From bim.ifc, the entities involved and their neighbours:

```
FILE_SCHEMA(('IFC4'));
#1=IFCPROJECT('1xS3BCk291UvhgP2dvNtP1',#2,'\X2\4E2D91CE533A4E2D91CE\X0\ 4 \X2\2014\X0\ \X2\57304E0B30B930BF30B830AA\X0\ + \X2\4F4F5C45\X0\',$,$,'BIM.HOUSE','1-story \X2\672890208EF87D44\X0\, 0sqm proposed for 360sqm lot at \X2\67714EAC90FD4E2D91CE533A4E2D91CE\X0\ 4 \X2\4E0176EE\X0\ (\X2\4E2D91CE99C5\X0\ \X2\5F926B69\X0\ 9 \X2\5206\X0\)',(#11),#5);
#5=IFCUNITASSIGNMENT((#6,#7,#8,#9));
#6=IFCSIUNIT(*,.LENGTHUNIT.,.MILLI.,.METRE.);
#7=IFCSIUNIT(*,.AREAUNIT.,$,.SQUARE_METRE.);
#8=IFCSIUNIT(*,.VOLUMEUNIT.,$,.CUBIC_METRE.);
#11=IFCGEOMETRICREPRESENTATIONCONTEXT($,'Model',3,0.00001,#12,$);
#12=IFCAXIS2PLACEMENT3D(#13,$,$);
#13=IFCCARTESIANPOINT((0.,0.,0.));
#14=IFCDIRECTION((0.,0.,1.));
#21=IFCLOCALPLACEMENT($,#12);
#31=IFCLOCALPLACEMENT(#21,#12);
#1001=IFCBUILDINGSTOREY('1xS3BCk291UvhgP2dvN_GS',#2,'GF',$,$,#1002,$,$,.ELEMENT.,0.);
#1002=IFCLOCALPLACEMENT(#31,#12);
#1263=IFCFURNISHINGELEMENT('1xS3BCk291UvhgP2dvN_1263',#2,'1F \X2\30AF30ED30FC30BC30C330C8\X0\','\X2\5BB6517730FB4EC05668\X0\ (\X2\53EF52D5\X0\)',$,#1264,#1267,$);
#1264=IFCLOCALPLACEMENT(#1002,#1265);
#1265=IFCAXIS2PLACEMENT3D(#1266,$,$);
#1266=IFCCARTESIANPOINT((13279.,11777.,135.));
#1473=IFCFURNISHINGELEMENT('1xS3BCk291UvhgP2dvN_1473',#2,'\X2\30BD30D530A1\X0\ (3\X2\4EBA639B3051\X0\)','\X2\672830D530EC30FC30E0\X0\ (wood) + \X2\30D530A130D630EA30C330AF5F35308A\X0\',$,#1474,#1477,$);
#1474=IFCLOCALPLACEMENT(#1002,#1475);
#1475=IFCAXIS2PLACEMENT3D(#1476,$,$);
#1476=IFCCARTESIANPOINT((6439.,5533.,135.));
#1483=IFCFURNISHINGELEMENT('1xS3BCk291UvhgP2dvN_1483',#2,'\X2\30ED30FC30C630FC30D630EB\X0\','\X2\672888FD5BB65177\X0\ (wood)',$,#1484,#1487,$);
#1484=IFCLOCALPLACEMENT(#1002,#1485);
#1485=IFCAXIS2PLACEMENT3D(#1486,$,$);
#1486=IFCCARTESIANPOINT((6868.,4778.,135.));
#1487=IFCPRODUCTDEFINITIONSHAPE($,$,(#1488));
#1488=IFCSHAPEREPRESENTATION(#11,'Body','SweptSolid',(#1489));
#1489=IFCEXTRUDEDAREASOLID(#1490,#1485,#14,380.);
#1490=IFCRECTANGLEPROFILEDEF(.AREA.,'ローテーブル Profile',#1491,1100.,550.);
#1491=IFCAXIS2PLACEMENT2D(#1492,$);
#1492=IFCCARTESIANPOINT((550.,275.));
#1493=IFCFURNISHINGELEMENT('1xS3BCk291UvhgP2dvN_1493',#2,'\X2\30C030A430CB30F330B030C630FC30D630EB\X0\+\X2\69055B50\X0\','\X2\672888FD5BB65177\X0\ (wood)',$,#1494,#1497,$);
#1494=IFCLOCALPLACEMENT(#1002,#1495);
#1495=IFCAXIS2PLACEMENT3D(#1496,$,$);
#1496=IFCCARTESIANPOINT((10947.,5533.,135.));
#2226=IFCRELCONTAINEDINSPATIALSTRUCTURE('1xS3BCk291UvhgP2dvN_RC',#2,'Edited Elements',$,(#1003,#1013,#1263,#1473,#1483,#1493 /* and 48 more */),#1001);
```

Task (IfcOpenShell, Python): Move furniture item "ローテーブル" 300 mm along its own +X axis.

```python
import ifcopenshell
import ifcopenshell.api.geometry
import ifcopenshell.util.placement
import ifcopenshell.util.unit

model = ifcopenshell.open("bim.ifc")
unit_scale = ifcopenshell.util.unit.calculate_unit_scale(model)

item = model.by_guid("1xS3BCk291UvhgP2dvN_1483")
matrix = ifcopenshell.util.placement.get_local_placement(item.ObjectPlacement)
matrix[:3, 3] += matrix[:3, 0] * 0.3 / unit_scale
ifcopenshell.api.geometry.edit_object_placement(model, product=item, matrix=matrix, is_si=False)

print(ifcopenshell.util.placement.get_local_placement(item.ObjectPlacement).round(3) + 0.0)

model.write("bim_rev.ifc")
```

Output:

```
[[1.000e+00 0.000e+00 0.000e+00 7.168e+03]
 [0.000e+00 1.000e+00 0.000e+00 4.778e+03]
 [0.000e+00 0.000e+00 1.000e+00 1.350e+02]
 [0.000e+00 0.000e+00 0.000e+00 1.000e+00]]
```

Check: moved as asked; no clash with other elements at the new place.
